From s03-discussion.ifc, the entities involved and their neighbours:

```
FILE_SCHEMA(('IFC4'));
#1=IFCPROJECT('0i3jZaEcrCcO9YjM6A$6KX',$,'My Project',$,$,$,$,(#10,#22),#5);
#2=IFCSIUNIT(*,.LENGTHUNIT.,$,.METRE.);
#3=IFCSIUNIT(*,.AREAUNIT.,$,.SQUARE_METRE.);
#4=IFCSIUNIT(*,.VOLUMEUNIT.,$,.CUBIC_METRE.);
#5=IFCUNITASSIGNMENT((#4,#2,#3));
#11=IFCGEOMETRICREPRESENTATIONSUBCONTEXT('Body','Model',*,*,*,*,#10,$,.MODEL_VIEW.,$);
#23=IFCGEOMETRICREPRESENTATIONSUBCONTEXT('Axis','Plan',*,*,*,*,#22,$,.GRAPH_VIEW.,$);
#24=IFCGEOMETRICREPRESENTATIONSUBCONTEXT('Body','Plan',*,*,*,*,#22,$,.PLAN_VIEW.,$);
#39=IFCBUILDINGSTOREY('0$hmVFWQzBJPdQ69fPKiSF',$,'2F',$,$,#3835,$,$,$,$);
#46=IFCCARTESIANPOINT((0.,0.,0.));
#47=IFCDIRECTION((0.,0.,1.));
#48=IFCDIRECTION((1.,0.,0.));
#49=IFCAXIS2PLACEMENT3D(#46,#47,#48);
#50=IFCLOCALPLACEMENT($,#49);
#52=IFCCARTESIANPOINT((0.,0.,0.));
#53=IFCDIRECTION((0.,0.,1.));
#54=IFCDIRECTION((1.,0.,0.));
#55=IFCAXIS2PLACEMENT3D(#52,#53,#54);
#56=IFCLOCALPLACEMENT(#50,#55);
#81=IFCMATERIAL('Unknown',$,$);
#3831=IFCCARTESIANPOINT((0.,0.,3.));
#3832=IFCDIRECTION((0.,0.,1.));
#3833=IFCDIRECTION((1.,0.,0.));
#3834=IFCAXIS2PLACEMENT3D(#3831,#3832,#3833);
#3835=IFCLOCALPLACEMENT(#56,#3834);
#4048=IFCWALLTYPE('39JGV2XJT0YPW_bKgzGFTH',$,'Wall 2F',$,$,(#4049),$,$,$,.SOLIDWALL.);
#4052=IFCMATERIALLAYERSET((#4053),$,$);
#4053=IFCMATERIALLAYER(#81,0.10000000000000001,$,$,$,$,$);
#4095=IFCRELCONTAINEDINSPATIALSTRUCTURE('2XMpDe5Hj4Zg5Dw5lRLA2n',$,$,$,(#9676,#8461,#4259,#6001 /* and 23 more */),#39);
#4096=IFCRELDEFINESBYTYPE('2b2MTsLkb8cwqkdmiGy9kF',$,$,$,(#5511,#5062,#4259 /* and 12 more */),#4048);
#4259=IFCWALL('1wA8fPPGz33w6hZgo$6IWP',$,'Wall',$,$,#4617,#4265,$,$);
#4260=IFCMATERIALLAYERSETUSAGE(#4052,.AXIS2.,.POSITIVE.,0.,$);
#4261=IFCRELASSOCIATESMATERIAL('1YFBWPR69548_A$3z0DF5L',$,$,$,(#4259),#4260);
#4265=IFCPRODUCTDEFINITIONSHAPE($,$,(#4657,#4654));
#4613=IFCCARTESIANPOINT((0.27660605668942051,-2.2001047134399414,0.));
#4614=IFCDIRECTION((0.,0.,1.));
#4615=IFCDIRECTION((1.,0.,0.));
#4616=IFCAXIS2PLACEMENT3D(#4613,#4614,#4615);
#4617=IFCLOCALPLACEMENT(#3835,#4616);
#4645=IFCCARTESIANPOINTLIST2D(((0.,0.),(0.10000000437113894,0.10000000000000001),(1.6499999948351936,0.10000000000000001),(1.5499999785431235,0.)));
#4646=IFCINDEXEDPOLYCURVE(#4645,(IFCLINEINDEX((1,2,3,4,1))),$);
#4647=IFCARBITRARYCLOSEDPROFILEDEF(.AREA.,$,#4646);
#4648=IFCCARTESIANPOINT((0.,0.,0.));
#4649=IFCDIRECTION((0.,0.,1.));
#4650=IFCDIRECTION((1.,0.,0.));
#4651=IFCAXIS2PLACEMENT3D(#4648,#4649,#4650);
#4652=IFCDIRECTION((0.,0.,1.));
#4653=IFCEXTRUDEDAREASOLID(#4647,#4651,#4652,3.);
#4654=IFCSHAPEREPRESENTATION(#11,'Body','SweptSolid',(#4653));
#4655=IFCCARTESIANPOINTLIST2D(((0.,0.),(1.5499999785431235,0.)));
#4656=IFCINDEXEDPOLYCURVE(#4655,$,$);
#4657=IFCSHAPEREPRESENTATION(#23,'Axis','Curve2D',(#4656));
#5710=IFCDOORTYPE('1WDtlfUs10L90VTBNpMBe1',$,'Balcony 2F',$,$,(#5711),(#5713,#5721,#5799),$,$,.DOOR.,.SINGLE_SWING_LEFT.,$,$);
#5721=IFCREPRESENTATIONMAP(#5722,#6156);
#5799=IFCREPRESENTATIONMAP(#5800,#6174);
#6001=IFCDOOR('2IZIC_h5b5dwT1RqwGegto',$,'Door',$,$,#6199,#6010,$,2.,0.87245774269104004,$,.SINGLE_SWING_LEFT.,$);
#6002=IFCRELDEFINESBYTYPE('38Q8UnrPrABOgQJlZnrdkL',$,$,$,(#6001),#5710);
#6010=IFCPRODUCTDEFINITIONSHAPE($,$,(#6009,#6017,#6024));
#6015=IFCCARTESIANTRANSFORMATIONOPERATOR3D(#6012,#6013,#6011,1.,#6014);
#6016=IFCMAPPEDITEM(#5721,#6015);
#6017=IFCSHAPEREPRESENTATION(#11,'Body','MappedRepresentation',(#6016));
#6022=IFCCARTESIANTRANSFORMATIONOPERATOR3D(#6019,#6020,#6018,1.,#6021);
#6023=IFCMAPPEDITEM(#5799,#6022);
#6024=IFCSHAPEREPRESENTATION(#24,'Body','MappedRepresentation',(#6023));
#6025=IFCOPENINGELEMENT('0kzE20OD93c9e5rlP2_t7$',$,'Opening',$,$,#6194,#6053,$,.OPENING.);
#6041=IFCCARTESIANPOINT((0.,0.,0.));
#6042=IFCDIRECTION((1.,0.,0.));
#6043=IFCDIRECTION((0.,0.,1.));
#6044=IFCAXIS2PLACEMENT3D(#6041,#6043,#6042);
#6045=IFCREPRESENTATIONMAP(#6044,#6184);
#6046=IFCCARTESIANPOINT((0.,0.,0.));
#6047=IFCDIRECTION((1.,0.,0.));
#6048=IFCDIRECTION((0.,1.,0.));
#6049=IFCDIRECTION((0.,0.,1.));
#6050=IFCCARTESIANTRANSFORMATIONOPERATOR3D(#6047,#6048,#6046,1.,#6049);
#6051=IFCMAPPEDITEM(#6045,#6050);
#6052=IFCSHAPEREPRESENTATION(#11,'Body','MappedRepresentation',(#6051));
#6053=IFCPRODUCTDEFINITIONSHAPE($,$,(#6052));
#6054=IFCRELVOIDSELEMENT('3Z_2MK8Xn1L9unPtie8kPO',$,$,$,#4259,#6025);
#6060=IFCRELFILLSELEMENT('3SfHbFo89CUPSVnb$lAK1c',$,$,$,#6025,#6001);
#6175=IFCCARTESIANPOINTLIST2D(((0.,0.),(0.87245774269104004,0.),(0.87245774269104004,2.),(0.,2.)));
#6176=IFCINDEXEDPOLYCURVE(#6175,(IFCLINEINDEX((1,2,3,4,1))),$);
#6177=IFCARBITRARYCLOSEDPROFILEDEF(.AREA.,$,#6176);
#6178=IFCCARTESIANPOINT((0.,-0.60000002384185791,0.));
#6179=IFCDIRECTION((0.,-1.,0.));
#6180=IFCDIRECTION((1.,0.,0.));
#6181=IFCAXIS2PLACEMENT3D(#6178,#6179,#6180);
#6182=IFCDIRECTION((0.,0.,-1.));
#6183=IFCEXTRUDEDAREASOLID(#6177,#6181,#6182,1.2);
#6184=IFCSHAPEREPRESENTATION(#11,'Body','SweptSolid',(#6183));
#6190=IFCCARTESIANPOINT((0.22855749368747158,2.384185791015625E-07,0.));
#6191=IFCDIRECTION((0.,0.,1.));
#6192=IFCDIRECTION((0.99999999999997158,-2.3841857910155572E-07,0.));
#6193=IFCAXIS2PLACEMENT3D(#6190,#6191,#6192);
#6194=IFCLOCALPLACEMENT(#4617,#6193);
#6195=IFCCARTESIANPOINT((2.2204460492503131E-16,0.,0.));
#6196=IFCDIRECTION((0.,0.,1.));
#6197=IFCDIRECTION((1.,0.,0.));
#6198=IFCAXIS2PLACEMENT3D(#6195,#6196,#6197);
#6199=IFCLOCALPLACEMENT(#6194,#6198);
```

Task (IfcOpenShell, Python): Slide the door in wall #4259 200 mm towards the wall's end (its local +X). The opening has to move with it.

```python
import ifcopenshell
import ifcopenshell.api.geometry
import ifcopenshell.util.placement
import ifcopenshell.util.unit

model = ifcopenshell.open("s03-discussion.ifc")
unit_scale = ifcopenshell.util.unit.calculate_unit_scale(model)

door = model.by_id(6001)
opening = door.FillsVoids[0].RelatingOpeningElement
wall = opening.VoidsElements[0].RelatingBuildingElement

wall_matrix = ifcopenshell.util.placement.get_local_placement(wall.ObjectPlacement)
shift = wall_matrix[:3, 0] * 0.2 / unit_scale
before = ifcopenshell.util.placement.get_local_placement(door.ObjectPlacement)[:3, 3].copy()

# The door is placed relative to its opening, so it follows when the opening moves.
matrix = ifcopenshell.util.placement.get_local_placement(opening.ObjectPlacement)
matrix[:3, 3] += shift
ifcopenshell.api.geometry.edit_object_placement(
    model, product=opening, matrix=matrix, is_si=False, should_transform_children=True
)

after = ifcopenshell.util.placement.get_local_placement(door.ObjectPlacement)[:3, 3]
print("door moved by", (after - before).round(3) + 0.0)

model.write("s03-discussion_v2.ifc")
```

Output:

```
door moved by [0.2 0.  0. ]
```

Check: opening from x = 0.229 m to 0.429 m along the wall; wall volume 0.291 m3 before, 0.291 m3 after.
